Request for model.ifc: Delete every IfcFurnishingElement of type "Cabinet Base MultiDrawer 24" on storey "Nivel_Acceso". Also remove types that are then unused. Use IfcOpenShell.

First a look at what the model holds.

```python
import ifcopenshell
import ifcopenshell.util.element

model = ifcopenshell.open("model.ifc")
print(model.schema)
storey = next(s for s in model.by_type("IfcBuildingStorey") if s.Name == "Nivel_Acceso")
furniture = [e for e in ifcopenshell.util.element.get_decomposition(storey) if e.is_a("IfcFurnishingElement")]
seen = {}
for e in furniture:
    element_type = ifcopenshell.util.element.get_type(e)
    name = element_type.Name if element_type not in (None, e) else None
    seen[name] = seen.get(name, 0) + 1
for name, count in sorted(seen.items(), key=str):
    print(count, "x", name)
```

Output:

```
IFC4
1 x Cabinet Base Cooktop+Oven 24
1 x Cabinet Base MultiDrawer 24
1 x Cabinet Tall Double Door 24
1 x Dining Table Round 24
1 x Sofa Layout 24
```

```python
import ifcopenshell
import ifcopenshell.api.root
import ifcopenshell.util.element

model = ifcopenshell.open("model.ifc")

storey = next(s for s in model.by_type("IfcBuildingStorey") if s.Name == "Nivel_Acceso")
furniture = [e for e in ifcopenshell.util.element.get_decomposition(storey) if e.is_a("IfcFurnishingElement")]
targets = [e for e in furniture if (t := ifcopenshell.util.element.get_type(e)) not in (None, e) and t.Name == "Cabinet Base MultiDrawer 24"]
types = {ifcopenshell.util.element.get_type(e) for e in targets} - {None, *targets}

for e in targets:
    ifcopenshell.api.root.remove_product(model, product=e)
print(len(targets), "removed")

unused = [t for t in types if not ifcopenshell.util.element.get_types(t)]
for t in unused:
    ifcopenshell.api.root.remove_product(model, product=t)
print(len(unused), "unused types removed")

model.write("model_edited.ifc")
```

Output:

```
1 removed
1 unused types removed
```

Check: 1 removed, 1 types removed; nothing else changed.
